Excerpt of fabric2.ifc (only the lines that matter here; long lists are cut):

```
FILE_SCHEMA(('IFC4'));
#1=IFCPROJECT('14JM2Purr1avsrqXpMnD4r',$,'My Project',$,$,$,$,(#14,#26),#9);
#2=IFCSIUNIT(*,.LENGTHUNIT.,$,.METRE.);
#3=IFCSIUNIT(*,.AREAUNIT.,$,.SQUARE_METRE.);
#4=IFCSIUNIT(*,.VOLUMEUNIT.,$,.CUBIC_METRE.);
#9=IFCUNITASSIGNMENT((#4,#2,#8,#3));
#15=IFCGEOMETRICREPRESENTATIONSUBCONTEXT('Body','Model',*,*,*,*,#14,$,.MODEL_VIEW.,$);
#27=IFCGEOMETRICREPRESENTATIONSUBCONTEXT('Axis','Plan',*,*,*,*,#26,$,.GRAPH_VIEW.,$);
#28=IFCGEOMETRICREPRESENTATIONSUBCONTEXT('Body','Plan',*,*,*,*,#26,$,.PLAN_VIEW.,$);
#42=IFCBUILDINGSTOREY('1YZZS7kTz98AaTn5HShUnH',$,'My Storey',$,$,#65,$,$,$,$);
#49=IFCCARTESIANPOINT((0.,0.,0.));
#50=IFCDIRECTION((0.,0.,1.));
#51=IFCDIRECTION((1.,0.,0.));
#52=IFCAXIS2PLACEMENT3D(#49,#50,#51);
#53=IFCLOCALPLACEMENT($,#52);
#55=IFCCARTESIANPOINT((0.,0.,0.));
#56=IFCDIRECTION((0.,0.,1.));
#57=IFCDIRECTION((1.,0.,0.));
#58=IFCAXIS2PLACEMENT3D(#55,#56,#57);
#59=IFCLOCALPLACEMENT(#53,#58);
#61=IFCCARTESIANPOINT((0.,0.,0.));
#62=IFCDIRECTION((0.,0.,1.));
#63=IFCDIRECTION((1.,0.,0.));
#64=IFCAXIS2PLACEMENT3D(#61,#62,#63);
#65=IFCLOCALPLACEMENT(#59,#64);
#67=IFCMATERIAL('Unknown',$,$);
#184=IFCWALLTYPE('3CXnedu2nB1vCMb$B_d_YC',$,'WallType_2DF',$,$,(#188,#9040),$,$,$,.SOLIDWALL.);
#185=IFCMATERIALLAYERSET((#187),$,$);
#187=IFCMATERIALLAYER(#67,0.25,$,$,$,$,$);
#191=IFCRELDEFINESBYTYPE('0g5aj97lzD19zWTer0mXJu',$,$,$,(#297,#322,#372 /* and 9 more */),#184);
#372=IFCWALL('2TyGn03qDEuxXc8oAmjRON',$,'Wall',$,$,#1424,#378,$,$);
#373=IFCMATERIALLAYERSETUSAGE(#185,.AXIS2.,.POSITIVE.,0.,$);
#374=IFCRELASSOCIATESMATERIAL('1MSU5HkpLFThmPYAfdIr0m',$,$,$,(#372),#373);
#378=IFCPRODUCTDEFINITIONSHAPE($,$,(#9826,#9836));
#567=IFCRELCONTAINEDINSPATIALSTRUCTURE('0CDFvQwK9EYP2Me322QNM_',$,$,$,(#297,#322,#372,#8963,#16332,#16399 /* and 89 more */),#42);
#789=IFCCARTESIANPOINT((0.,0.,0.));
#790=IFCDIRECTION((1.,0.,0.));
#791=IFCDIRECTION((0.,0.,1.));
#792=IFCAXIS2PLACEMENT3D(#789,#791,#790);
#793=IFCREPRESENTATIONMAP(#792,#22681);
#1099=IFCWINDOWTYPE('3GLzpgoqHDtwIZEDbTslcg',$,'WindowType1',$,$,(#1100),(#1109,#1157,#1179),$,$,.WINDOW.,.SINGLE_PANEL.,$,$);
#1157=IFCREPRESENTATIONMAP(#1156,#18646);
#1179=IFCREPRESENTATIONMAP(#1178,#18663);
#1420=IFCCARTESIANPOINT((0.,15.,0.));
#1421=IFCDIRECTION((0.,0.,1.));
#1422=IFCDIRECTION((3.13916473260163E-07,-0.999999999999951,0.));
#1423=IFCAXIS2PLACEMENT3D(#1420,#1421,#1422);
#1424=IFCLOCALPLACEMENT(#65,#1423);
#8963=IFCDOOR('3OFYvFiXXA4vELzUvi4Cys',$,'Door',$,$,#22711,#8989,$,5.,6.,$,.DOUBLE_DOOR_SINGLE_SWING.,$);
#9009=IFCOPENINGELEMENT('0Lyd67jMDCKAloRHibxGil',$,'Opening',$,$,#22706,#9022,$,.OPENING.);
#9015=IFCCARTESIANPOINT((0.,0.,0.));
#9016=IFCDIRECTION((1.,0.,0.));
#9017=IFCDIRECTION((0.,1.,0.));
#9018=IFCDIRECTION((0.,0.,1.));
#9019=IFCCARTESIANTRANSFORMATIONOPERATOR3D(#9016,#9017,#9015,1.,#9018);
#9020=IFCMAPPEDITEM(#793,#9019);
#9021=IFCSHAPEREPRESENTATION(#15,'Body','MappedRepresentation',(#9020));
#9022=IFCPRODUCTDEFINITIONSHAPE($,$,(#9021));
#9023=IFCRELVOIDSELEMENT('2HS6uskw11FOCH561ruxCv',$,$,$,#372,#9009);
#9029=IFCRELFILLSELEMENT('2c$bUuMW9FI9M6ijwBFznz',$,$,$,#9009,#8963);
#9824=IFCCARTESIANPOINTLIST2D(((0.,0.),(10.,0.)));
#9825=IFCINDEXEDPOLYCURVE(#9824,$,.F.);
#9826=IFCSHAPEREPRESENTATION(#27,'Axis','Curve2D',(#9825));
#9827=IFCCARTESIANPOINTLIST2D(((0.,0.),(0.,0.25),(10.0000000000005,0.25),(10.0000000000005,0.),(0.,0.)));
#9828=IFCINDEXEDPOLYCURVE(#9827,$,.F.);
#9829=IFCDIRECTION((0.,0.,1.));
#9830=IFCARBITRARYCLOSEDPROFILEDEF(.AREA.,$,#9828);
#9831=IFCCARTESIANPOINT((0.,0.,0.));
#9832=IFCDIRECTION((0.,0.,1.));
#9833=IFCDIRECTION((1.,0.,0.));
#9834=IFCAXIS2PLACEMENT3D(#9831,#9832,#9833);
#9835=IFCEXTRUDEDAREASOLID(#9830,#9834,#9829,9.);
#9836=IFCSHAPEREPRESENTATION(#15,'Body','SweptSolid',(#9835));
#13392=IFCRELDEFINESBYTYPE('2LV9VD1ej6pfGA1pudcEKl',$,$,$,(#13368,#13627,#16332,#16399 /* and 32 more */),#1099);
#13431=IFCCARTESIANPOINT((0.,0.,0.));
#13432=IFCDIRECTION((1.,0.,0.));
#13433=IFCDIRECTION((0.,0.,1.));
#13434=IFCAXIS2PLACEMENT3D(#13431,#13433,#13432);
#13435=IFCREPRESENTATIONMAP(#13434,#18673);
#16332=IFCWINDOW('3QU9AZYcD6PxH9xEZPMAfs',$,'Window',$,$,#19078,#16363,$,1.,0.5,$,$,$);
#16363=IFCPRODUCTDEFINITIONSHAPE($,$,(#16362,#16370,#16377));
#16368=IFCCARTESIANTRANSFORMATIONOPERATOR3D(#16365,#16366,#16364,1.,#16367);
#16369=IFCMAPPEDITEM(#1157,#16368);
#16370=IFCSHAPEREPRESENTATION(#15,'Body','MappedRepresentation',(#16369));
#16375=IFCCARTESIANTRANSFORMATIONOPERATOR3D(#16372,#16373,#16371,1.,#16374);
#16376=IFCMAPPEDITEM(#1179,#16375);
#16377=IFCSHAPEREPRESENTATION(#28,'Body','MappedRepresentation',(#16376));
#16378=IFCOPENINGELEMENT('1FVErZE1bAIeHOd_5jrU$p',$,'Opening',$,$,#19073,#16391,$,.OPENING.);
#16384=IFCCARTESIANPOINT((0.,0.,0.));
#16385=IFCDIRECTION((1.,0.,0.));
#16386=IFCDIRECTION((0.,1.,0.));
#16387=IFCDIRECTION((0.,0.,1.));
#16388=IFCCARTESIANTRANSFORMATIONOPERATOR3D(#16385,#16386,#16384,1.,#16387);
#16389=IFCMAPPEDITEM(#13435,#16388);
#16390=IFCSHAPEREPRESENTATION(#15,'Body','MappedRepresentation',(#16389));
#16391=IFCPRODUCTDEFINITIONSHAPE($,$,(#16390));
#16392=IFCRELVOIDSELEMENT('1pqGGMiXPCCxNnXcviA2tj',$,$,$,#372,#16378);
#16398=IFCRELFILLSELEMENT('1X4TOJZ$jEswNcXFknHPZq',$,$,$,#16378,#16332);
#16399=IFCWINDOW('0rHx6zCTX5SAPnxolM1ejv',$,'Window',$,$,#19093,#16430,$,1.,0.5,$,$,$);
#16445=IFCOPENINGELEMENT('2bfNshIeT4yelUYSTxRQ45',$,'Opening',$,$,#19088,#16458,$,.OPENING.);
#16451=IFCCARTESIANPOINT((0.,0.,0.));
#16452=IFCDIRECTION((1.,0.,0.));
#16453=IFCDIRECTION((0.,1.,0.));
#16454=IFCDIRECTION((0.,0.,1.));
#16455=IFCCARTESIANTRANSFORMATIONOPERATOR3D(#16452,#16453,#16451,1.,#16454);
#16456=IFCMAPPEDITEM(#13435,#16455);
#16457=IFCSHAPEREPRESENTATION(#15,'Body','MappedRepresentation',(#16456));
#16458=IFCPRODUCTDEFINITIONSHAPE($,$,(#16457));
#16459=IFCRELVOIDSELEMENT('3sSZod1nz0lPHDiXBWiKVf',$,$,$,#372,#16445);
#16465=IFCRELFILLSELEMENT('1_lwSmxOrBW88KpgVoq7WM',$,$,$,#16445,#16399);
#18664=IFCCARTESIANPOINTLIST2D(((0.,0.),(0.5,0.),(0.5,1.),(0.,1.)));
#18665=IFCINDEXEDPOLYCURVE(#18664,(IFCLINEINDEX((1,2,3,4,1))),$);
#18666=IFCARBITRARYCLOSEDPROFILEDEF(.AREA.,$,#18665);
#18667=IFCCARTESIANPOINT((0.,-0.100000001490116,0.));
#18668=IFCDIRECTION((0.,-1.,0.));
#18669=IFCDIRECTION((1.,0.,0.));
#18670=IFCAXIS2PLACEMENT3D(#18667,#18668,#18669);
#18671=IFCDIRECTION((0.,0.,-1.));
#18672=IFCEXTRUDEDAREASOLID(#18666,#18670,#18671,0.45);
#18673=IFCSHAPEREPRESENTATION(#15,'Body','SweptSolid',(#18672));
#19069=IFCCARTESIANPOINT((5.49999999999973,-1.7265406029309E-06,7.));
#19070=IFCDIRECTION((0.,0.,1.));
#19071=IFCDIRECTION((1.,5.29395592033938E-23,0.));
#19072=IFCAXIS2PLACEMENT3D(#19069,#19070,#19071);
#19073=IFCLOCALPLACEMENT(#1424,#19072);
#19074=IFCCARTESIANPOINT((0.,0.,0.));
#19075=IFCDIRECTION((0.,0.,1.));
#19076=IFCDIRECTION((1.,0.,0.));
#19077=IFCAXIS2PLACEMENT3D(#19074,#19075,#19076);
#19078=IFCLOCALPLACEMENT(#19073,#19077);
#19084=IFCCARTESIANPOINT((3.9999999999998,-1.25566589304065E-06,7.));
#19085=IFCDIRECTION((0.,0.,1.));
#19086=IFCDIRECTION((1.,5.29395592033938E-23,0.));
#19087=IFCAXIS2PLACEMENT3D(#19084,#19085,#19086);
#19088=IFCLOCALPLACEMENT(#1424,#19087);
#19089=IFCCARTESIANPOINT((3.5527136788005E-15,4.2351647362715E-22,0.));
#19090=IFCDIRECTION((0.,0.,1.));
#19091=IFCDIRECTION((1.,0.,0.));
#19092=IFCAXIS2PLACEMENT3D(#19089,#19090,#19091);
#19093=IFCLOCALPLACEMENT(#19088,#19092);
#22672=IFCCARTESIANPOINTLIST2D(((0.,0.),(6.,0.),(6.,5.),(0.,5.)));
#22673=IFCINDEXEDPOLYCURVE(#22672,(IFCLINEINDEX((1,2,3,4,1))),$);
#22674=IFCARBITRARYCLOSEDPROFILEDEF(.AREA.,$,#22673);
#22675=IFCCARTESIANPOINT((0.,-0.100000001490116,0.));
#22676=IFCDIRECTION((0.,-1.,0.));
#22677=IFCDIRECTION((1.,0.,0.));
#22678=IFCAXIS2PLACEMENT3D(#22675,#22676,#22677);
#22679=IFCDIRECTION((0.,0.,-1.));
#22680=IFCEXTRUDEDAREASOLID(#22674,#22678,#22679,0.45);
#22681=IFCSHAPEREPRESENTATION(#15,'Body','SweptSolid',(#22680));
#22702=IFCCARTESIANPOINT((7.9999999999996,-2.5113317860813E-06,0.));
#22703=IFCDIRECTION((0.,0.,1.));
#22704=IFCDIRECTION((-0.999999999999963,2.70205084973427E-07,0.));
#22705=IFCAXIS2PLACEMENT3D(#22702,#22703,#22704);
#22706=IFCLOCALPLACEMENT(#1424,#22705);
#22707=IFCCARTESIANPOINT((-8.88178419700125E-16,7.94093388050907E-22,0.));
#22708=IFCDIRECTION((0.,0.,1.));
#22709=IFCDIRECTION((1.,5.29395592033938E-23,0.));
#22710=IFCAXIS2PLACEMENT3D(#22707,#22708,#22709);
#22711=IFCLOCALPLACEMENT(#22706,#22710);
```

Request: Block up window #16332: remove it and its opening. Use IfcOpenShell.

```python
import ifcopenshell
import ifcopenshell.api.feature
import ifcopenshell.api.root
import ifcopenshell.geom
import ifcopenshell.util.shape

model = ifcopenshell.open("fabric2.ifc")
settings = ifcopenshell.geom.settings()


def volume(element):
    """Net volume in cubic metres, openings subtracted."""
    shape = ifcopenshell.geom.create_shape(settings, element)
    return ifcopenshell.util.shape.get_volume(shape.geometry)


window = model.by_guid("3QU9AZYcD6PxH9xEZPMAfs")
opening = window.FillsVoids[0].RelatingOpeningElement
wall = opening.VoidsElements[0].RelatingBuildingElement
before = volume(wall)

ifcopenshell.api.root.remove_product(model, product=window)
ifcopenshell.api.feature.remove_feature(model, feature=opening)

after = volume(wall)

print(f"wall volume {before:.3f} -> {after:.3f} m3")

model.write("fabric2_updated.ifc")
```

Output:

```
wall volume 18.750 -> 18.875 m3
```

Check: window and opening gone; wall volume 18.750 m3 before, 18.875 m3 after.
